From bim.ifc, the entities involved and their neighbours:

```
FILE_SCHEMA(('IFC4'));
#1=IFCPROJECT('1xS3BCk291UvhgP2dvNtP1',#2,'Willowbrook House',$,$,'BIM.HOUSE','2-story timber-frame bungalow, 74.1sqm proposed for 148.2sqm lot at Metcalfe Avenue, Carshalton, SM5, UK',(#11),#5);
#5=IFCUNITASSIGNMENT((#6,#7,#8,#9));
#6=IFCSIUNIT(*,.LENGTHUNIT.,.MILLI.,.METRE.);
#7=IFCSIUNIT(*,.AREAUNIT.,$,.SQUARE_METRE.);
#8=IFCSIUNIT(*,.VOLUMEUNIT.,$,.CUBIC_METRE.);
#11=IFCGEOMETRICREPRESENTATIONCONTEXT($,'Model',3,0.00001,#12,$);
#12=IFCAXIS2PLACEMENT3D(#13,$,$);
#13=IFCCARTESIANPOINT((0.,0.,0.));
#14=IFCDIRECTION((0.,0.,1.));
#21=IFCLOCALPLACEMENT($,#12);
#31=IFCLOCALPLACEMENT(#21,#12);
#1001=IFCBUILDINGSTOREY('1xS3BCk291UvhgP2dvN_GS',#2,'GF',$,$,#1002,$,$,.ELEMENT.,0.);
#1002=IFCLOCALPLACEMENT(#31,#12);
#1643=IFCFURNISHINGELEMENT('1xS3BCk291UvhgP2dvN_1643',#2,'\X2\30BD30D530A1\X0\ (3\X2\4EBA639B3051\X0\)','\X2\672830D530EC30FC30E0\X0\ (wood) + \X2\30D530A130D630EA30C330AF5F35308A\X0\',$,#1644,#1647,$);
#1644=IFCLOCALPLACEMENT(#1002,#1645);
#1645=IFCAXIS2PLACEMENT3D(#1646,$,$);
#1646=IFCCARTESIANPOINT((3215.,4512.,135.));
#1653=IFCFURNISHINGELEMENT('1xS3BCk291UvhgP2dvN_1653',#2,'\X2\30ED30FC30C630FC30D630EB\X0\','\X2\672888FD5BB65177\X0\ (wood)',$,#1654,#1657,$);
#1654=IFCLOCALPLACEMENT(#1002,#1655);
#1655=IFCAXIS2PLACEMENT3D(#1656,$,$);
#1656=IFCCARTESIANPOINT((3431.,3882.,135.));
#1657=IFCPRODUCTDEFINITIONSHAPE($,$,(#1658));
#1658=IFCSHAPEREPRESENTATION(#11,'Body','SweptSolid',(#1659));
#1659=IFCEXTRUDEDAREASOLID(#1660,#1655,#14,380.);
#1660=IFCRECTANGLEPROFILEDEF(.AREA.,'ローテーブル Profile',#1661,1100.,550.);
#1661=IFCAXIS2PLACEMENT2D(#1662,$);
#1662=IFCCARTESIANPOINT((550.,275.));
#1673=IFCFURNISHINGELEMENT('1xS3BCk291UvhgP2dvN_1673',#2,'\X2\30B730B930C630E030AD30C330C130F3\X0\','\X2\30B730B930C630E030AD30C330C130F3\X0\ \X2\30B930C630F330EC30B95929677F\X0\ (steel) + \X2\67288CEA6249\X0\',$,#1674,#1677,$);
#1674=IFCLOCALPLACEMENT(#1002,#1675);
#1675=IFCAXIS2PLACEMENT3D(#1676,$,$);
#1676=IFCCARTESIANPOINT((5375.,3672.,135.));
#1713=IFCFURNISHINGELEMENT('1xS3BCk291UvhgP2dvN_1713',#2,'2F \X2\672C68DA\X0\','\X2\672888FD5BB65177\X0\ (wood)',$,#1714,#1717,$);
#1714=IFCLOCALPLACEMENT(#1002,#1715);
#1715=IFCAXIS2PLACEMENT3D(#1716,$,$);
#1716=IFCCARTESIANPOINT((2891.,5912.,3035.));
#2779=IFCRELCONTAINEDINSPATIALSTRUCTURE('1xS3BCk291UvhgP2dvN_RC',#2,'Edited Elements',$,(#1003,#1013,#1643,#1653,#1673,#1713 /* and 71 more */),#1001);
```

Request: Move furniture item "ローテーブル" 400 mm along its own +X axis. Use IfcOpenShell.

```python
import ifcopenshell
import ifcopenshell.api.geometry
import ifcopenshell.util.placement
import ifcopenshell.util.unit

model = ifcopenshell.open("bim.ifc")
unit_scale = ifcopenshell.util.unit.calculate_unit_scale(model)

item = model.by_guid("1xS3BCk291UvhgP2dvN_1653")
matrix = ifcopenshell.util.placement.get_local_placement(item.ObjectPlacement)
matrix[:3, 3] += matrix[:3, 0] * 0.4 / unit_scale
ifcopenshell.api.geometry.edit_object_placement(model, product=item, matrix=matrix, is_si=False)

print(ifcopenshell.util.placement.get_local_placement(item.ObjectPlacement).round(3) + 0.0)

model.write("bim_updated.ifc")
```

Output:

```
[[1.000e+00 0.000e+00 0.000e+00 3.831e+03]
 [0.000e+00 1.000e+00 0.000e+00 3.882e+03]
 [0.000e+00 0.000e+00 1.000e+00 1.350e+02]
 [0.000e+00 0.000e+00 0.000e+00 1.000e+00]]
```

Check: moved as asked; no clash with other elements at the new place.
